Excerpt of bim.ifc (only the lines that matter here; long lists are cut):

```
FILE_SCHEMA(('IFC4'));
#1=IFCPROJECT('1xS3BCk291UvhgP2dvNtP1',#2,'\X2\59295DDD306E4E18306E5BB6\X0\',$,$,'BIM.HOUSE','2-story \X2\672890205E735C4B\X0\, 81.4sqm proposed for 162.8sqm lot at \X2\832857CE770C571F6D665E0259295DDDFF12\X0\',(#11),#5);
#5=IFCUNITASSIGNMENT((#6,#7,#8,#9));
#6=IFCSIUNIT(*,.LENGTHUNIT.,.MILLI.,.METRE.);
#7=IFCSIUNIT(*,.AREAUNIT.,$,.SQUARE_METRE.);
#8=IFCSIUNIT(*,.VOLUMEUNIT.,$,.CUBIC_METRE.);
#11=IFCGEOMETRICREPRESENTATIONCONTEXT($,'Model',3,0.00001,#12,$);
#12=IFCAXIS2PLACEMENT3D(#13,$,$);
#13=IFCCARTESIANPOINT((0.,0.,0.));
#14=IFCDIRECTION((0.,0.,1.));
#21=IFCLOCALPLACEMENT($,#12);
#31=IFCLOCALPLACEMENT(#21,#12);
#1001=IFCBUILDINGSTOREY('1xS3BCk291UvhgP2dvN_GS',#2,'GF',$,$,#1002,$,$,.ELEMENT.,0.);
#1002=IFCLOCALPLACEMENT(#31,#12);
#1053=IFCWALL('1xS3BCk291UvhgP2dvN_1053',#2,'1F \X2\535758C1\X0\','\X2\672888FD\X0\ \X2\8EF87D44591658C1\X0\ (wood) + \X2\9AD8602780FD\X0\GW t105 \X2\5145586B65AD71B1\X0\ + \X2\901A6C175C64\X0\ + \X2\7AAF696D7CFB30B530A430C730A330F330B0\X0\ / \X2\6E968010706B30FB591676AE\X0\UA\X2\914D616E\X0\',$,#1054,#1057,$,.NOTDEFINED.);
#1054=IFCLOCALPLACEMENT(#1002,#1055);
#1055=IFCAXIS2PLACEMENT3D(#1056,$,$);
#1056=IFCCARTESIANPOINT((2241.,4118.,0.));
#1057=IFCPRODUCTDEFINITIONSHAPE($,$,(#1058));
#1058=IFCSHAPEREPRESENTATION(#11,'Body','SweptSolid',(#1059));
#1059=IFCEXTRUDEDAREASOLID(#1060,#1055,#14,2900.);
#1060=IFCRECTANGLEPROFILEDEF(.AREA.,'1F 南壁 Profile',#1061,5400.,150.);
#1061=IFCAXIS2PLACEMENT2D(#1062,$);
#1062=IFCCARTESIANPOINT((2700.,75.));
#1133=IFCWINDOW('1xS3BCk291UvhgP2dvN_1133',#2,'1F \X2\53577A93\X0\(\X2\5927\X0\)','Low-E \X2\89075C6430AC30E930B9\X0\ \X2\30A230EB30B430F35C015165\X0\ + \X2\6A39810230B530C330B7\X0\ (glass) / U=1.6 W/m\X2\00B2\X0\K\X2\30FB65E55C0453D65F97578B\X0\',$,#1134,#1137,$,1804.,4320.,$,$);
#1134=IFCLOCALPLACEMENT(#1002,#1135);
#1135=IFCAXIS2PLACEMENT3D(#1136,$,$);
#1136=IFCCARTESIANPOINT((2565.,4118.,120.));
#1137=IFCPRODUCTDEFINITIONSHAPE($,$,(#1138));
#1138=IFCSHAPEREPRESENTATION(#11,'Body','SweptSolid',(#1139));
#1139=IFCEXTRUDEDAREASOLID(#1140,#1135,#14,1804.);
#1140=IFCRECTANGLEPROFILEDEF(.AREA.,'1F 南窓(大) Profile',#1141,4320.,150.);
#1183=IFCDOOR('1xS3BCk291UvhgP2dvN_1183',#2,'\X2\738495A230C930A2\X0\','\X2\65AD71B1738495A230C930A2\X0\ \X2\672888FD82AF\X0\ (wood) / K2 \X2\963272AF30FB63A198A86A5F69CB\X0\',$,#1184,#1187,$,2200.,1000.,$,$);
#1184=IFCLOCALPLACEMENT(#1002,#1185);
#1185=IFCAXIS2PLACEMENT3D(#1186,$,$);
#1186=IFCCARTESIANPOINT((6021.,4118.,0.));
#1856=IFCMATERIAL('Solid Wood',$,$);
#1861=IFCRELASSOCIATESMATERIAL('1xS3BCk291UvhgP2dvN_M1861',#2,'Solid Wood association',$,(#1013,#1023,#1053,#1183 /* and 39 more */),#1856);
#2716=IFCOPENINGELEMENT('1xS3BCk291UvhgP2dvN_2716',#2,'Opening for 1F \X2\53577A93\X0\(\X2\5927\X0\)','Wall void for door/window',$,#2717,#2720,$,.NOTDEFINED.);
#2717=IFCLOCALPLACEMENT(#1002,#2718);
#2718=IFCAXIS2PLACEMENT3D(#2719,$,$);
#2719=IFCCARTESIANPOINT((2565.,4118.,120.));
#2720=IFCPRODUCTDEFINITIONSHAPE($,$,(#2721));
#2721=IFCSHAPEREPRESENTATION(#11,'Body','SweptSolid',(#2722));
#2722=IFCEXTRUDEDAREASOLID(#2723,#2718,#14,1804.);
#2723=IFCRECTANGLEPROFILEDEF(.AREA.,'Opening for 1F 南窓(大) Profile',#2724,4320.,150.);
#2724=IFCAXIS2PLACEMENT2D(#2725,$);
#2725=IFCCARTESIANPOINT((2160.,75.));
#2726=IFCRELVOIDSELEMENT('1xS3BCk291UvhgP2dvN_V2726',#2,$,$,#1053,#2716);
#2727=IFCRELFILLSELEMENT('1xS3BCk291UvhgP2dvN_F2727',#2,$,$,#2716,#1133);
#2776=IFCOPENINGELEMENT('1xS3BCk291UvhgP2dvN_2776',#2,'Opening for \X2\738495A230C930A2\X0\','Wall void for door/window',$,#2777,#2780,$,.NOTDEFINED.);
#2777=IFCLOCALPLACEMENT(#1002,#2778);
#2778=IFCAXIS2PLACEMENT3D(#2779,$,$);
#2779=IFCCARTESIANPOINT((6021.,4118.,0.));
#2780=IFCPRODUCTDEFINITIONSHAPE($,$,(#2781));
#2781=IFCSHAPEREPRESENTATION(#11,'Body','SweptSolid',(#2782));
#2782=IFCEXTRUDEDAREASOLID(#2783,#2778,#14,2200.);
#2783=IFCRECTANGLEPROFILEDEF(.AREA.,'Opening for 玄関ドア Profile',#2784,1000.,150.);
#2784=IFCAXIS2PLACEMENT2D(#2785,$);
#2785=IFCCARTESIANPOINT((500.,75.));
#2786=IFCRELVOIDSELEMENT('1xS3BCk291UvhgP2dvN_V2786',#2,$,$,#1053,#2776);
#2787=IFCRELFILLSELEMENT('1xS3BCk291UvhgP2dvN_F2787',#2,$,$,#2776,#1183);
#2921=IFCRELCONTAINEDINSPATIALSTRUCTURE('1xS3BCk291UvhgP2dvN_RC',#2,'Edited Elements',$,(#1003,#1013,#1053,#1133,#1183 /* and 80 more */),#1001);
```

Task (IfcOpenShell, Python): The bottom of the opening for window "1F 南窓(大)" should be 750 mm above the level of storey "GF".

```python
import numpy as np
import ifcopenshell
import ifcopenshell.api.geometry
import ifcopenshell.geom
import ifcopenshell.util.element
import ifcopenshell.util.placement
import ifcopenshell.util.shape
import ifcopenshell.util.unit

model = ifcopenshell.open("bim.ifc")
unit_scale = ifcopenshell.util.unit.calculate_unit_scale(model)

window = model.by_guid("1xS3BCk291UvhgP2dvN_1133")
opening = window.FillsVoids[0].RelatingOpeningElement
storey = ifcopenshell.util.element.get_container(window, ifc_class="IfcBuildingStorey")
level = ifcopenshell.util.placement.get_local_placement(storey.ObjectPlacement)[2, 3]

# The opening's origin need not be at the sill, so measure its lowest point.
shape = ifcopenshell.geom.create_shape(ifcopenshell.geom.settings(), opening)
bottom = ifcopenshell.util.shape.get_shape_bottom_elevation(shape, shape.geometry) / unit_scale
dz = level + 750.0 - bottom

shift = np.array([0.0, 0.0, dz])
# The window is not placed relative to its opening, so move both.
for product in (opening, window):
    matrix = ifcopenshell.util.placement.get_local_placement(product.ObjectPlacement)
    matrix[:3, 3] += shift
    ifcopenshell.api.geometry.edit_object_placement(model, product=product, matrix=matrix, is_si=False)

print(f"moved by {dz * unit_scale:+.3f} m")

model.write("bim_edited.ifc")
```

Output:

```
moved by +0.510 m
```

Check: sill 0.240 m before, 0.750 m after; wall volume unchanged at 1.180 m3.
